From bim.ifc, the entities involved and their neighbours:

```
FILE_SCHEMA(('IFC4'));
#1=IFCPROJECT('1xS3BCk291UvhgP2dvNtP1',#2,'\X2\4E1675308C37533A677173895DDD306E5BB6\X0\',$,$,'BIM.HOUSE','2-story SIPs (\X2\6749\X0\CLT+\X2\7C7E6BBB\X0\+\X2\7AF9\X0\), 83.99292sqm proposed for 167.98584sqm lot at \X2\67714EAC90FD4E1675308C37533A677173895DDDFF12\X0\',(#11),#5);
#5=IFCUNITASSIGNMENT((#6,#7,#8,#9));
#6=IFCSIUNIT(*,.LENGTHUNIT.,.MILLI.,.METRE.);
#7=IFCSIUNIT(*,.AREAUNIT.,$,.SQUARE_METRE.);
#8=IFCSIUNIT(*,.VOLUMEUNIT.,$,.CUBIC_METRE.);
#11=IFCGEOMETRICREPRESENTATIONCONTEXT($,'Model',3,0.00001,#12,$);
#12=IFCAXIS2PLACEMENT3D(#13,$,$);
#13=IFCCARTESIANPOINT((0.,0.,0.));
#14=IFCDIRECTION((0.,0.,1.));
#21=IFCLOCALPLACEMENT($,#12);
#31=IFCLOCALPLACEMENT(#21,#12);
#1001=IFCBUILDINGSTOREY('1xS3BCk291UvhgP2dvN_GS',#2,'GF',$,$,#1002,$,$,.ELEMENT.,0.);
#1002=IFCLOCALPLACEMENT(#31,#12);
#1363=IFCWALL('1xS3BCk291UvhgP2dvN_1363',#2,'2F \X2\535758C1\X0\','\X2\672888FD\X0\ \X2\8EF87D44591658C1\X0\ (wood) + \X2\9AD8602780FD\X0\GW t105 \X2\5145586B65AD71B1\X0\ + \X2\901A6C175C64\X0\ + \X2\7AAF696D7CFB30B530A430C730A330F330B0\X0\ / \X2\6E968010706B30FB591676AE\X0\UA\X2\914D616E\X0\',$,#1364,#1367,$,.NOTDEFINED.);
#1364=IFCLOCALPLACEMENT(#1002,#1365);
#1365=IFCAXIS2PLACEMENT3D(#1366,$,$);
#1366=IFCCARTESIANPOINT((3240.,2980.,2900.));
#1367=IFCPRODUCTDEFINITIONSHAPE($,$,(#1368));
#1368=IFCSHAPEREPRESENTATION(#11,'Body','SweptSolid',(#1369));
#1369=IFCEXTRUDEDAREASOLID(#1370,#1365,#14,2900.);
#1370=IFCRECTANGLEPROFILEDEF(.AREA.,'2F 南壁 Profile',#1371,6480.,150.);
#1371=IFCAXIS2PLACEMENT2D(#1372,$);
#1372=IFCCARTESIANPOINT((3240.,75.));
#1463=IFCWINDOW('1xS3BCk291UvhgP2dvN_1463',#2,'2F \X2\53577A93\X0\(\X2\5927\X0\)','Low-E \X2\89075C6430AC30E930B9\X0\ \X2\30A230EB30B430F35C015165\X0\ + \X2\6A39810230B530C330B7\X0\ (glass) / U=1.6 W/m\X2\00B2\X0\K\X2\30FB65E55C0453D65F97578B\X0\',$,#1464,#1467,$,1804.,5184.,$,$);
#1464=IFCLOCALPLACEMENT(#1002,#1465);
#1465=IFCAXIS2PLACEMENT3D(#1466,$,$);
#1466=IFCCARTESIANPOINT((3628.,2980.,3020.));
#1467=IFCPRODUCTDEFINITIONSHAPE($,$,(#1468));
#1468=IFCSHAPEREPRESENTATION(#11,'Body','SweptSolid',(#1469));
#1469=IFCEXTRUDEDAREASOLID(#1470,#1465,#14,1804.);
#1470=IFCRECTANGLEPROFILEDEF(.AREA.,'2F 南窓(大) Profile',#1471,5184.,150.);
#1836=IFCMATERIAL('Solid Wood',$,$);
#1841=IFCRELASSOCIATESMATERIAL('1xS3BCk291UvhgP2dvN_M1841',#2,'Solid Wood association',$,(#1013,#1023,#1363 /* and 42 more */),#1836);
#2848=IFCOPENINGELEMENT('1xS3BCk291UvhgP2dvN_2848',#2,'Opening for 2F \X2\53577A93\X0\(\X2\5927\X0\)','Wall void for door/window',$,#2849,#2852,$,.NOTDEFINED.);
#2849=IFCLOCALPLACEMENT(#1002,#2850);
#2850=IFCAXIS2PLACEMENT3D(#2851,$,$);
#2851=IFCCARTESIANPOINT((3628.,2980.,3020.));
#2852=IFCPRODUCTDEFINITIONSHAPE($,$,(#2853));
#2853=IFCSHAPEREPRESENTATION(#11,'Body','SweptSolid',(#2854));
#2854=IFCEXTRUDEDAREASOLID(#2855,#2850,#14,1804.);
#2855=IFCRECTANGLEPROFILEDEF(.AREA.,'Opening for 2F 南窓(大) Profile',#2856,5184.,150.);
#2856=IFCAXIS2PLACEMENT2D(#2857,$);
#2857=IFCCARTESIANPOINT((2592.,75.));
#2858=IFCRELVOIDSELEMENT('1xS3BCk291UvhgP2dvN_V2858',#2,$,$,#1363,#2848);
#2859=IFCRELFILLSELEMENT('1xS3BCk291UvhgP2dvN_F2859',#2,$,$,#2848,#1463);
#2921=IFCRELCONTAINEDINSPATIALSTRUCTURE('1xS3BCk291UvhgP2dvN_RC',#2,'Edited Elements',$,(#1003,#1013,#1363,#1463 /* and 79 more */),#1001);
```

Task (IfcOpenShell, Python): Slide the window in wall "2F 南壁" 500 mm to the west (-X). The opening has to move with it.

```python
import ifcopenshell
import ifcopenshell.api.geometry
import ifcopenshell.util.placement
import ifcopenshell.util.unit

model = ifcopenshell.open("bim.ifc")
unit_scale = ifcopenshell.util.unit.calculate_unit_scale(model)

window = model.by_id(1463)
opening = window.FillsVoids[0].RelatingOpeningElement
wall = opening.VoidsElements[0].RelatingBuildingElement

wall_matrix = ifcopenshell.util.placement.get_local_placement(wall.ObjectPlacement)
shift = wall_matrix[:3, 0] * -0.5 / unit_scale
before = ifcopenshell.util.placement.get_local_placement(window.ObjectPlacement)[:3, 3].copy()

# The window is not placed relative to its opening, so move both.
for product in (opening, window):
    matrix = ifcopenshell.util.placement.get_local_placement(product.ObjectPlacement)
    matrix[:3, 3] += shift
    ifcopenshell.api.geometry.edit_object_placement(model, product=product, matrix=matrix, is_si=False)

after = ifcopenshell.util.placement.get_local_placement(window.ObjectPlacement)[:3, 3]
print("window moved by", (after - before).round(3) + 0.0)

model.write("bim_v2.ifc")
```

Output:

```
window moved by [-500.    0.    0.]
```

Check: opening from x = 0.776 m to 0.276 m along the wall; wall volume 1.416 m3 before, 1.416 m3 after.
